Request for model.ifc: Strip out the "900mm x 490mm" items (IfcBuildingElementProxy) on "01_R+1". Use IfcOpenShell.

First a look at what the model holds.

```python
import ifcopenshell
import ifcopenshell.util.element

model = ifcopenshell.open("model.ifc")
print(model.schema)
storey = next(s for s in model.by_type("IfcBuildingStorey") if s.Name == "01_R+1")
proxies = [e for e in ifcopenshell.util.element.get_decomposition(storey) if e.is_a("IfcBuildingElementProxy")]
seen = {}
for e in proxies:
    element_type = ifcopenshell.util.element.get_type(e)
    name = element_type.Name if element_type not in (None, e) else None
    seen[name] = seen.get(name, 0) + 1
for name, count in sorted(seen.items(), key=str):
    print(count, "x", name)
```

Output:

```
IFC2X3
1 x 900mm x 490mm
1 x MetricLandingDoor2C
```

```python
import ifcopenshell
import ifcopenshell.api.root
import ifcopenshell.util.element

model = ifcopenshell.open("model.ifc")

storey = next(s for s in model.by_type("IfcBuildingStorey") if s.Name == "01_R+1")
proxies = [e for e in ifcopenshell.util.element.get_decomposition(storey) if e.is_a("IfcBuildingElementProxy")]
targets = [e for e in proxies if (t := ifcopenshell.util.element.get_type(e)) not in (None, e) and t.Name == "900mm x 490mm"]

for e in targets:
    ifcopenshell.api.root.remove_product(model, product=e)
print(len(targets), "removed")

model.write("model_updated.ifc")
```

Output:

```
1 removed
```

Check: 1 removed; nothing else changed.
